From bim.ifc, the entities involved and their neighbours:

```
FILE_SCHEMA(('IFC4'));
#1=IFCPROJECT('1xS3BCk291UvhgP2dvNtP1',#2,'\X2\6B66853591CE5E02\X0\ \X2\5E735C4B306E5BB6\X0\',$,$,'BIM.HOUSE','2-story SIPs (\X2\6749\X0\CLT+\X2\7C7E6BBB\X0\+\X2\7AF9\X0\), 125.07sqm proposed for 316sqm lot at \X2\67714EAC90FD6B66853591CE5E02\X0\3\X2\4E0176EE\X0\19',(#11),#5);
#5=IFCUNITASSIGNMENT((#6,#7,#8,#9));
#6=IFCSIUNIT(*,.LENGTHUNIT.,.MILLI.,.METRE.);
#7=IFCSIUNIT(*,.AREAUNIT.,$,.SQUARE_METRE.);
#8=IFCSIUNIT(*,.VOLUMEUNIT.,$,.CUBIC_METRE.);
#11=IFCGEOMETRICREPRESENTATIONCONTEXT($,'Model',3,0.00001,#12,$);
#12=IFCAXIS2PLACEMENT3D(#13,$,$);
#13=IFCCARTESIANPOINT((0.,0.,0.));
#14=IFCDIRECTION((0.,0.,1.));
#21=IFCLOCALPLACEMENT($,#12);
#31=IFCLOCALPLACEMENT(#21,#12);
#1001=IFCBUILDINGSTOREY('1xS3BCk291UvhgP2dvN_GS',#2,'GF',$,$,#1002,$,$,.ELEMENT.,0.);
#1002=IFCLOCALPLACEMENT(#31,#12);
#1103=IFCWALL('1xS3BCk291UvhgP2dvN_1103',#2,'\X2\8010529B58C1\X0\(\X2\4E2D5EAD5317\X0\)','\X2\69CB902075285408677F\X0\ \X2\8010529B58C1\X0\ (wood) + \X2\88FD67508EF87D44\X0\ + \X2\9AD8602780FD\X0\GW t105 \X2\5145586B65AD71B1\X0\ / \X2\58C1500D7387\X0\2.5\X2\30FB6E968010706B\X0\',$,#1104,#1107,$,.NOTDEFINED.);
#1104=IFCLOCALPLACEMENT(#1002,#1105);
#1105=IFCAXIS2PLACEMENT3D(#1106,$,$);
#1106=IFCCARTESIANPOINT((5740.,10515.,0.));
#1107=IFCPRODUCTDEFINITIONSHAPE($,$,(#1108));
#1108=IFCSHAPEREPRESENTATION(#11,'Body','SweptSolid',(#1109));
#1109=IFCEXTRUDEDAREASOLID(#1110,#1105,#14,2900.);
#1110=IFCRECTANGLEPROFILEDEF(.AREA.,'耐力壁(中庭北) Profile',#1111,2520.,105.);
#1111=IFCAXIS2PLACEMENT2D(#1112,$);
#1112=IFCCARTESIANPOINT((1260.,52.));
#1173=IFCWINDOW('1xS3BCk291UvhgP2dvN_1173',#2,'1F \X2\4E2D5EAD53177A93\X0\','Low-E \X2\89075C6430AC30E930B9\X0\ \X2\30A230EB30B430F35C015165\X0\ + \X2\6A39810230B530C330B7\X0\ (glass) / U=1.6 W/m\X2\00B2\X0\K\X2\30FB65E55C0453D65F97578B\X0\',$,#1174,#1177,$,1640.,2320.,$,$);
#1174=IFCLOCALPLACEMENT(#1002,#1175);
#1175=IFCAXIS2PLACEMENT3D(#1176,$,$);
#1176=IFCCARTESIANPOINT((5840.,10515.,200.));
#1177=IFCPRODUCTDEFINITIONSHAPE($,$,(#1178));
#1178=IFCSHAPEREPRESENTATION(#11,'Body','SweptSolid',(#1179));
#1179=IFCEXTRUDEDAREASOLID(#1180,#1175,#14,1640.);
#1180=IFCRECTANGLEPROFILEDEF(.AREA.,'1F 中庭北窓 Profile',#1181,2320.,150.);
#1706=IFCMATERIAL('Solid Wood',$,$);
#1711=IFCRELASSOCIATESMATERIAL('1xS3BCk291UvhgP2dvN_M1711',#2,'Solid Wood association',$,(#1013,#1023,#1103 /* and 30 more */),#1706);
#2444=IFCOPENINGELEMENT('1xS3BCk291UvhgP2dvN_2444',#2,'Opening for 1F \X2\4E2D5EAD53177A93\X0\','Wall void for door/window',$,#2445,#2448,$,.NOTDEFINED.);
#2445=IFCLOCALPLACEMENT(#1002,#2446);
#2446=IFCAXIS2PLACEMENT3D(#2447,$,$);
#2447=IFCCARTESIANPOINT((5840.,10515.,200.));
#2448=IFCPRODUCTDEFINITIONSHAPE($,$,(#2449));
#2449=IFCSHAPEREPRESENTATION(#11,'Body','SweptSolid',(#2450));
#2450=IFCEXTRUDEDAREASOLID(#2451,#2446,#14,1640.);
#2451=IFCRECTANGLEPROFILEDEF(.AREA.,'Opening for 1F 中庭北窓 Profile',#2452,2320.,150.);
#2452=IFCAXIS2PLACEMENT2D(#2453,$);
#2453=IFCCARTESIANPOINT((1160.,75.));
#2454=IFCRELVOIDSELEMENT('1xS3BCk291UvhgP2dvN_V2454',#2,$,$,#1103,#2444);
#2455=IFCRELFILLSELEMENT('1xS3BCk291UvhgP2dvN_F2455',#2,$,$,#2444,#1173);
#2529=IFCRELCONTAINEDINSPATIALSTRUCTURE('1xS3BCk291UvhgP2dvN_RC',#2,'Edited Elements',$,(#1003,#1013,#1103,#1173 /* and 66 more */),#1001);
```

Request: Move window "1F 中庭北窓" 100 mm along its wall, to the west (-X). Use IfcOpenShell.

```python
import ifcopenshell
import ifcopenshell.api.geometry
import ifcopenshell.util.placement

model = ifcopenshell.open("bim.ifc")

window = model.by_guid("1xS3BCk291UvhgP2dvN_1173")
opening = window.FillsVoids[0].RelatingOpeningElement
wall = opening.VoidsElements[0].RelatingBuildingElement

wall_matrix = ifcopenshell.util.placement.get_local_placement(wall.ObjectPlacement)
shift = wall_matrix[:3, 0] * -100.0
before = ifcopenshell.util.placement.get_local_placement(window.ObjectPlacement)[:3, 3].copy()

# The window is not placed relative to its opening, so move both.
for product in (opening, window):
    matrix = ifcopenshell.util.placement.get_local_placement(product.ObjectPlacement)
    matrix[:3, 3] += shift
    ifcopenshell.api.geometry.edit_object_placement(model, product=product, matrix=matrix, is_si=False)

after = ifcopenshell.util.placement.get_local_placement(window.ObjectPlacement)[:3, 3]
print("window moved by", (after - before).round(3) + 0.0)

model.write("bim_v2.ifc")
```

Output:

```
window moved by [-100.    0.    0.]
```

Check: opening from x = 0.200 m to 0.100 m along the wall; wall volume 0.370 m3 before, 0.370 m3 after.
